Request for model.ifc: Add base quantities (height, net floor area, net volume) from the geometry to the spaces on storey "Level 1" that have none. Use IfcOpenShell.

First a look at what the model holds.

```python
import ifcopenshell
import ifcopenshell.util.element
import ifcopenshell.util.unit

model = ifcopenshell.open("model.ifc")
print(model.schema)
for unit_type in ("LENGTHUNIT", "AREAUNIT", "VOLUMEUNIT"):
    print(unit_type, ifcopenshell.util.unit.calculate_unit_scale(model, unit_type))
storey = next(s for s in model.by_type("IfcBuildingStorey") if s.Name == "Level 1")
spaces = [e for e in ifcopenshell.util.element.get_decomposition(storey) if e.is_a("IfcSpace")]
for e in sorted(spaces, key=lambda e: e.id()):
    print(e.id(), e.is_a(), e.Name, list(ifcopenshell.util.element.get_psets(e, qtos_only=True)), sep=" | ")
```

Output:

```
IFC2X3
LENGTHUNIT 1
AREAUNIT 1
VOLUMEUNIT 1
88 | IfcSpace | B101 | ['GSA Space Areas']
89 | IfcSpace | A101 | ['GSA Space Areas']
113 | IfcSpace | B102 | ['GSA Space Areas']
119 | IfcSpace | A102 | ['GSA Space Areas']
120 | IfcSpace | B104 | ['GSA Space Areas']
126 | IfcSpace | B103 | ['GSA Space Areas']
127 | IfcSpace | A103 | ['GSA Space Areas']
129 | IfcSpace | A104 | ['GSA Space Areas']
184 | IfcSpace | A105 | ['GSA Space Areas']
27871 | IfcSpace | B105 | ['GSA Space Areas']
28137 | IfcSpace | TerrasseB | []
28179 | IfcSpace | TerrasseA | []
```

```python
import ifcopenshell
import ifcopenshell.api.pset
import ifcopenshell.geom
import ifcopenshell.util.element
import ifcopenshell.util.shape
import ifcopenshell.util.unit

model = ifcopenshell.open("model.ifc")
unit_scale = ifcopenshell.util.unit.calculate_unit_scale(model)
area_scale = ifcopenshell.util.unit.calculate_unit_scale(model, "AREAUNIT")
volume_scale = ifcopenshell.util.unit.calculate_unit_scale(model, "VOLUMEUNIT")
settings = ifcopenshell.geom.settings()

storey = next(s for s in model.by_type("IfcBuildingStorey") if s.Name == "Level 1")
spaces = [e for e in ifcopenshell.util.element.get_decomposition(storey) if e.is_a("IfcSpace")]

for e in sorted(spaces, key=lambda e: e.id()):
    if ifcopenshell.util.element.get_psets(e, qtos_only=True, should_inherit=False):
        continue
    # Geometry comes back in metres, in the element's own axes.
    shape = ifcopenshell.geom.create_shape(settings, e)
    values = {
        "Height": ifcopenshell.util.shape.get_z(shape.geometry) / unit_scale,
        "NetFloorArea": ifcopenshell.util.shape.get_footprint_area(shape.geometry) / area_scale,
        "NetVolume": ifcopenshell.util.shape.get_volume(shape.geometry) / volume_scale,
    }
    qto = ifcopenshell.api.pset.add_qto(model, product=e, name="BaseQuantities")
    ifcopenshell.api.pset.edit_qto(model, qto=qto, properties=values)
    print(e.id(), {k: round(v, 3) for k, v in values.items()})

model.write("model_v2.ifc")
```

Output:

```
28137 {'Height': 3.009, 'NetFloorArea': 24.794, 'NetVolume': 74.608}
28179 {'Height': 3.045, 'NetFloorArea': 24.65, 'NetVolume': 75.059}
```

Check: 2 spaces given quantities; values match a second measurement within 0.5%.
